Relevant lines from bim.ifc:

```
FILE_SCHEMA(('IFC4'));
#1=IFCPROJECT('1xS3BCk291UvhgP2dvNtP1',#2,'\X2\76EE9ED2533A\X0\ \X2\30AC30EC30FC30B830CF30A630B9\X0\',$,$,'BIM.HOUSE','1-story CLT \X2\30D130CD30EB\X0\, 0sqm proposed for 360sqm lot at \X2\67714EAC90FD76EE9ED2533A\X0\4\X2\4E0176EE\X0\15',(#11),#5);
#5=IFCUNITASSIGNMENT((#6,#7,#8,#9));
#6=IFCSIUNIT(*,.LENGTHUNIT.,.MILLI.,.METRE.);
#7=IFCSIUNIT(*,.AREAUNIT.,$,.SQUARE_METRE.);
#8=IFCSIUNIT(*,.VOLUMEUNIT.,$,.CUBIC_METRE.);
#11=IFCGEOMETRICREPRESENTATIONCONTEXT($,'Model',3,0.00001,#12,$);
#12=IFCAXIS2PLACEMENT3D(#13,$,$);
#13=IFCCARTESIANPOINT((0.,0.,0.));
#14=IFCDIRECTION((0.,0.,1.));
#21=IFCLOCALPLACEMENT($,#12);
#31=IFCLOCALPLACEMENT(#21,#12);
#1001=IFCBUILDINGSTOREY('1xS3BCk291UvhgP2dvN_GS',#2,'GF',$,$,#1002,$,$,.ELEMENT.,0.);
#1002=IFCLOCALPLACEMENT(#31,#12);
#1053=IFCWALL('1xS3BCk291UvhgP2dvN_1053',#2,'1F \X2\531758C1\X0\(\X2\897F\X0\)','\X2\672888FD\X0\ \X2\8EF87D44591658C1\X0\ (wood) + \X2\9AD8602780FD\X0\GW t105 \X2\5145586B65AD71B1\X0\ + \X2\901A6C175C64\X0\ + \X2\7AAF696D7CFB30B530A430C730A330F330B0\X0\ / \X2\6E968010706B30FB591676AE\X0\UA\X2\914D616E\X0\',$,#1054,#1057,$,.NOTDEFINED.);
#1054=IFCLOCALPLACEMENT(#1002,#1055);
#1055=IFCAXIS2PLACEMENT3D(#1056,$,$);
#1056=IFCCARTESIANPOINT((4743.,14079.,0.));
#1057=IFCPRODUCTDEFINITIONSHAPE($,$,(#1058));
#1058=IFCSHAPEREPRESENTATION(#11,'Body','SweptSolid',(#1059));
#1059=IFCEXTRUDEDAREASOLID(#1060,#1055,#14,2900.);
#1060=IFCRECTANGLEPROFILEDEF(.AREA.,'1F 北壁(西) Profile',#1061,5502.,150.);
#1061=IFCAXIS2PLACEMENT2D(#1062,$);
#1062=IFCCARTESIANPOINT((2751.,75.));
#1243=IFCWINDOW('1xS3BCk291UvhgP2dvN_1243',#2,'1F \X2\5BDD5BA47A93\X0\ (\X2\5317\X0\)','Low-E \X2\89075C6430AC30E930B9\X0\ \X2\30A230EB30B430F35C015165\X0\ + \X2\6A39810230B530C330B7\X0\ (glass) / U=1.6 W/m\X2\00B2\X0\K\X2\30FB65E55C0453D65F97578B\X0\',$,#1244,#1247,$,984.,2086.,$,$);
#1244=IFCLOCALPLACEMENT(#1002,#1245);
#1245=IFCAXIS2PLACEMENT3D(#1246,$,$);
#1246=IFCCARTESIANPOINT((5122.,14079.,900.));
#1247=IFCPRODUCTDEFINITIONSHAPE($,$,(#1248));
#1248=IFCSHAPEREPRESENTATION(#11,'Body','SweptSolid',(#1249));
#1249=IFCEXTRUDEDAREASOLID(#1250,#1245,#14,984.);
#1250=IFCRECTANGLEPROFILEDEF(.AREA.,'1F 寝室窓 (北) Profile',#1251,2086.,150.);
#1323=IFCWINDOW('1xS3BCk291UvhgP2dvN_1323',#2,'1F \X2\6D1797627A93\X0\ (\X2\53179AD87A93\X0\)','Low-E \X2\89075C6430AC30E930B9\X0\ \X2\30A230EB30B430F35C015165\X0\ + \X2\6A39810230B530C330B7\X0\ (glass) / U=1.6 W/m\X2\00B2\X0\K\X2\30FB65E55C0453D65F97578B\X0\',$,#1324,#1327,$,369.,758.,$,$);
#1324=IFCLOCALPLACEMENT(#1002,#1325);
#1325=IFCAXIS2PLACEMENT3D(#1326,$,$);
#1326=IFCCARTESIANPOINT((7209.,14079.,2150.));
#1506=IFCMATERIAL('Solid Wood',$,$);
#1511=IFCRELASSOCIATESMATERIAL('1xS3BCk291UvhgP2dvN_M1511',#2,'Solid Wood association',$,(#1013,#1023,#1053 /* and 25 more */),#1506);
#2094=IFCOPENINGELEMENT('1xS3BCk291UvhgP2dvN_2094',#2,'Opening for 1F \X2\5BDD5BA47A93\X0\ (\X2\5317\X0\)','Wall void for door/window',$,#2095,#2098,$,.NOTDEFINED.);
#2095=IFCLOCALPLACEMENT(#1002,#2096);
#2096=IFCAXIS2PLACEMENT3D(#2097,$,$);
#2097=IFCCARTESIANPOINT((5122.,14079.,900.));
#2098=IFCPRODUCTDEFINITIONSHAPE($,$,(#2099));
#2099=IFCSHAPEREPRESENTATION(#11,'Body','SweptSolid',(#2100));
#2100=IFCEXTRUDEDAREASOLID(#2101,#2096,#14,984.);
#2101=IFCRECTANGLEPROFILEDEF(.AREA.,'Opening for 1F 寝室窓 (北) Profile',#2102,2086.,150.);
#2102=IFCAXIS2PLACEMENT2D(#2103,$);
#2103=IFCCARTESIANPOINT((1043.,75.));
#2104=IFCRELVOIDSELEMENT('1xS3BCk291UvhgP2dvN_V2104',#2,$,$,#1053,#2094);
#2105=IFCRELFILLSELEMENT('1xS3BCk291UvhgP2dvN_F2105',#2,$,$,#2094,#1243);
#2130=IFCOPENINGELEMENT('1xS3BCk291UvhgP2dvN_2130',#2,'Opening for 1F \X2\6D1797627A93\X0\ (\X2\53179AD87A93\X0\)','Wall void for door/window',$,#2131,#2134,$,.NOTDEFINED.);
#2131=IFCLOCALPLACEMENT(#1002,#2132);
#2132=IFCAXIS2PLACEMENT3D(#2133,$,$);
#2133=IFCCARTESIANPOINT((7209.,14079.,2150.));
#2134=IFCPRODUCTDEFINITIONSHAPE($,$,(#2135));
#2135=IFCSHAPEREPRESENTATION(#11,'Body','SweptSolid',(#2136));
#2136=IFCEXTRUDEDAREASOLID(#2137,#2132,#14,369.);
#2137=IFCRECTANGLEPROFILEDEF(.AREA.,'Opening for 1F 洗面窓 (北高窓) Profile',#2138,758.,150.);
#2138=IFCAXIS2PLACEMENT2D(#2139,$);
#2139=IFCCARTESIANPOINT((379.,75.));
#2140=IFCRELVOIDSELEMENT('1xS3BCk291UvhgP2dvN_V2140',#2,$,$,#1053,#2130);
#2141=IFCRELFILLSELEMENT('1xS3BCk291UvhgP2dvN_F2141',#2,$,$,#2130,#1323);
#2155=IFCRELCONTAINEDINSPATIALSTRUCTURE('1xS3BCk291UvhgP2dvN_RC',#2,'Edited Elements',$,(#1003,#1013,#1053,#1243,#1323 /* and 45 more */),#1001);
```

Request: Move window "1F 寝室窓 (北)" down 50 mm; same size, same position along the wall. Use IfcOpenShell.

```python
import numpy as np
import ifcopenshell
import ifcopenshell.api.geometry
import ifcopenshell.util.placement
import ifcopenshell.util.unit

model = ifcopenshell.open("bim.ifc")
unit_scale = ifcopenshell.util.unit.calculate_unit_scale(model)

window = model.by_id(1243)
opening = window.FillsVoids[0].RelatingOpeningElement
dz = -50.0

shift = np.array([0.0, 0.0, dz])
# The window is not placed relative to its opening, so move both.
for product in (opening, window):
    matrix = ifcopenshell.util.placement.get_local_placement(product.ObjectPlacement)
    matrix[:3, 3] += shift
    ifcopenshell.api.geometry.edit_object_placement(model, product=product, matrix=matrix, is_si=False)

print(f"moved by {dz * unit_scale:+.3f} m")

model.write("bim-out.ifc")
```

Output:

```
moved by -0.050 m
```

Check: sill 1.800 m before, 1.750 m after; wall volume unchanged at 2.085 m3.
